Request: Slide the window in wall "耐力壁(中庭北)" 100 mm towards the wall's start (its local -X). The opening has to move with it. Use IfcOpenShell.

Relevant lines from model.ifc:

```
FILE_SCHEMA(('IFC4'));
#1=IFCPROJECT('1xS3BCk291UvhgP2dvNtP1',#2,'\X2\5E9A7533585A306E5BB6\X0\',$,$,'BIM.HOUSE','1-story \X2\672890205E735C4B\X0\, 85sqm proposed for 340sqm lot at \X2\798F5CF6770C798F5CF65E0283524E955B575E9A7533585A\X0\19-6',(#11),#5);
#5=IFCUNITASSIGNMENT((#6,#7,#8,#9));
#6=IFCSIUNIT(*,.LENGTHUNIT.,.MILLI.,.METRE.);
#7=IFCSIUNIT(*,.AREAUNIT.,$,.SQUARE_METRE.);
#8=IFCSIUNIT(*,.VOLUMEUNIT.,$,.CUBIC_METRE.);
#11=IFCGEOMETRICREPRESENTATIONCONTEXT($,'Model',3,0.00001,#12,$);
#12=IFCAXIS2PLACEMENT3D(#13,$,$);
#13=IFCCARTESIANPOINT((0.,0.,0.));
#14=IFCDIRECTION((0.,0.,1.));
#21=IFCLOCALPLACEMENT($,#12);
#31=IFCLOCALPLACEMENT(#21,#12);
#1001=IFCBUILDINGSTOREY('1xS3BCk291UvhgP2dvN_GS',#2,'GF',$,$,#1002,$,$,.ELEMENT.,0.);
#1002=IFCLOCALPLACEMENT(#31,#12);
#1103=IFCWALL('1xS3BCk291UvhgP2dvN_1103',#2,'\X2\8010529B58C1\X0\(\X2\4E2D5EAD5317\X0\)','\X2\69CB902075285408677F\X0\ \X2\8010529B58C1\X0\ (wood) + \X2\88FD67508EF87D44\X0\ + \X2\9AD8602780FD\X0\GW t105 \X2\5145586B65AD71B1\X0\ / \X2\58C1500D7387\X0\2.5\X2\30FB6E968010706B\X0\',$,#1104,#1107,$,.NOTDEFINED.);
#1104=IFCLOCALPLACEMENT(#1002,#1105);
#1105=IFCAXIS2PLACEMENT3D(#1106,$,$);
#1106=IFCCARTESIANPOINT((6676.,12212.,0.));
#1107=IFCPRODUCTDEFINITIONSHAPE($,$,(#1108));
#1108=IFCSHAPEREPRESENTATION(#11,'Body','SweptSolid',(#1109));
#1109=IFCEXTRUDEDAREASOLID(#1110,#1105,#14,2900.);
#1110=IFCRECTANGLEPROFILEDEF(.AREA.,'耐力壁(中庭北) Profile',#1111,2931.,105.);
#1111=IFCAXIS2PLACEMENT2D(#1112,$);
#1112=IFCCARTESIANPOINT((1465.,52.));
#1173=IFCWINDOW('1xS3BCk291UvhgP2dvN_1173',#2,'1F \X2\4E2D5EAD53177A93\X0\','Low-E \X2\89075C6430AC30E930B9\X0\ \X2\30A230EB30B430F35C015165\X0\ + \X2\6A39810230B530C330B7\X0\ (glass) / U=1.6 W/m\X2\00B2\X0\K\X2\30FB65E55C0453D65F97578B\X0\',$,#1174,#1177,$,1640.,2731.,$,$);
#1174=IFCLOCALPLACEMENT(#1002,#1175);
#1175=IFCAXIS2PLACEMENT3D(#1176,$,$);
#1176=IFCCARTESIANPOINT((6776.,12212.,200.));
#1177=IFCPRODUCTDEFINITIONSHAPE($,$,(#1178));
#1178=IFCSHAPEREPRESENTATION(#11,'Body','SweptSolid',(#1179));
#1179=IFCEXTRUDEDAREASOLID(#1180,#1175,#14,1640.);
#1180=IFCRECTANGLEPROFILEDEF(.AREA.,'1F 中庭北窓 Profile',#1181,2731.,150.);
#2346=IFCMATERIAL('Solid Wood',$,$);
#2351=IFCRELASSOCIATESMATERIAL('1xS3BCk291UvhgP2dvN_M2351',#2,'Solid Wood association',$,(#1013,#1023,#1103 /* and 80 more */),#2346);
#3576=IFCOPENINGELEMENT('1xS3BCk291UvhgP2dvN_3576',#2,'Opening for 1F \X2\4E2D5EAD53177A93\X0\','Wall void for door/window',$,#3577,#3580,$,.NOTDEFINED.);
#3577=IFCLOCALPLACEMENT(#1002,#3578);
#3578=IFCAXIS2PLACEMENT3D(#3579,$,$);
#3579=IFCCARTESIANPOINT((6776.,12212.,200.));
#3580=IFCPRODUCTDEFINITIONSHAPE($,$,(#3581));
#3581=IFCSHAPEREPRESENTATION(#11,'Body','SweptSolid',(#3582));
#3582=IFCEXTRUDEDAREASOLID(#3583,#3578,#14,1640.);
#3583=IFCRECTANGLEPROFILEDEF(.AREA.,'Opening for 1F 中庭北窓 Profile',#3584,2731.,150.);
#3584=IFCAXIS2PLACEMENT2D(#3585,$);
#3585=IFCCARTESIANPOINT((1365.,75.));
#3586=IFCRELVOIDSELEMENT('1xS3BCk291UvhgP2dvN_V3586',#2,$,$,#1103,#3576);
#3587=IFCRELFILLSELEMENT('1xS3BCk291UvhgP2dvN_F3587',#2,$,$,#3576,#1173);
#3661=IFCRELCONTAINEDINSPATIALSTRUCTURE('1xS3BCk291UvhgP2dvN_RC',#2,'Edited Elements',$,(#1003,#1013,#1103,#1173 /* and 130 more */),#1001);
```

```python
import ifcopenshell
import ifcopenshell.api.geometry
import ifcopenshell.util.placement

model = ifcopenshell.open("model.ifc")

window = model.by_guid("1xS3BCk291UvhgP2dvN_1173")
opening = window.FillsVoids[0].RelatingOpeningElement
wall = opening.VoidsElements[0].RelatingBuildingElement

wall_matrix = ifcopenshell.util.placement.get_local_placement(wall.ObjectPlacement)
shift = wall_matrix[:3, 0] * -100.0
before = ifcopenshell.util.placement.get_local_placement(window.ObjectPlacement)[:3, 3].copy()

# The window is not placed relative to its opening, so move both.
for product in (opening, window):
    matrix = ifcopenshell.util.placement.get_local_placement(product.ObjectPlacement)
    matrix[:3, 3] += shift
    ifcopenshell.api.geometry.edit_object_placement(model, product=product, matrix=matrix, is_si=False)

after = ifcopenshell.util.placement.get_local_placement(window.ObjectPlacement)[:3, 3]
print("window moved by", (after - before).round(3) + 0.0)

model.write("model_v2.ifc")
```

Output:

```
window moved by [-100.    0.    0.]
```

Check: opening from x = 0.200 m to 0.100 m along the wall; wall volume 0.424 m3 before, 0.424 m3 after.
